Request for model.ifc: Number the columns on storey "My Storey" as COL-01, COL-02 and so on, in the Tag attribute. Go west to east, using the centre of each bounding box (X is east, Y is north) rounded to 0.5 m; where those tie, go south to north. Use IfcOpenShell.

First a look at what the model holds.

```python
import ifcopenshell
import ifcopenshell.util.element
import ifcopenshell.util.placement

model = ifcopenshell.open("model.ifc")
print(model.schema)
storey = next(s for s in model.by_type("IfcBuildingStorey") if s.Name == "My Storey")
columns = [e for e in ifcopenshell.util.element.get_decomposition(storey) if e.is_a("IfcColumn")]
for e in sorted(columns, key=lambda e: e.id()):
    origin = ifcopenshell.util.placement.get_local_placement(e.ObjectPlacement)[:3, 3]
    print(e.id(), e.Tag, e.Name, origin.round(2) + 0.0, sep=" | ")
```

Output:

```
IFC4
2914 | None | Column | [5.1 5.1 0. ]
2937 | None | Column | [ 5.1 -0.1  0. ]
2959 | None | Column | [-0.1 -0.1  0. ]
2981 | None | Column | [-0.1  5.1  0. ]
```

```python
import ifcopenshell
import ifcopenshell.geom
import ifcopenshell.util.element
import ifcopenshell.util.shape

model = ifcopenshell.open("model.ifc")
settings = ifcopenshell.geom.settings()
settings.set("use-world-coords", True)


def centre(element):
    shape = ifcopenshell.geom.create_shape(settings, element)
    return ifcopenshell.util.shape.get_bbox_centroid(shape.geometry)


storey = next(s for s in model.by_type("IfcBuildingStorey") if s.Name == "My Storey")
columns = [e for e in ifcopenshell.util.element.get_decomposition(storey) if e.is_a("IfcColumn")]

# Insertion points can sit at a corner or the storey origin, so sort by the geometry (in metres).
centres = {e: centre(e) for e in columns}
columns.sort(key=lambda e: (round(centres[e][0] / 0.5), centres[e][1]))

for i, e in enumerate(columns, start=1):
    number = f"COL-{i:02d}"
    e.Tag = number
    print(e.id(), number)

model.write("model-out.ifc")
```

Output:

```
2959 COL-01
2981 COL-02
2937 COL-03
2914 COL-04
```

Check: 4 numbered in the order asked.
